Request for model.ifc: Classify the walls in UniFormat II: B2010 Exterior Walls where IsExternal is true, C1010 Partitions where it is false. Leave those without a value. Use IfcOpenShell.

First a look at what the model holds.

```python
import ifcopenshell
import ifcopenshell.util.element

model = ifcopenshell.open("model.ifc")
print(model.schema)
print("classifications:", [c.Name for c in model.by_type("IfcClassification")])
values = [ifcopenshell.util.element.get_pset(e, "Pset_WallCommon", "IsExternal") for e in model.by_type("IfcWall")]
for value in (True, False, None):
    print("IsExternal", value, values.count(value))
```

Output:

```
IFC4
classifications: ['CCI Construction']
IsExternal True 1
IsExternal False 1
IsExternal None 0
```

```python
import ifcopenshell
import ifcopenshell.api.classification
import ifcopenshell.util.element

model = ifcopenshell.open("model.ifc")

system = ifcopenshell.api.classification.add_classification(model, classification="UniFormat II")

walls = model.by_type("IfcWall")
external = {e: ifcopenshell.util.element.get_pset(e, "Pset_WallCommon", "IsExternal") for e in walls}
for flag, code, name in ((True, "B2010", "Exterior Walls"), (False, "C1010", "Partitions")):
    products = [e for e in walls if external[e] is flag]
    ifcopenshell.api.classification.add_reference(
        model, products=products, classification=system, identification=code, name=name
    )
    print(code, len(products))

model.write("model_rev.ifc")
```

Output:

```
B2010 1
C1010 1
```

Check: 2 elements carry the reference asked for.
